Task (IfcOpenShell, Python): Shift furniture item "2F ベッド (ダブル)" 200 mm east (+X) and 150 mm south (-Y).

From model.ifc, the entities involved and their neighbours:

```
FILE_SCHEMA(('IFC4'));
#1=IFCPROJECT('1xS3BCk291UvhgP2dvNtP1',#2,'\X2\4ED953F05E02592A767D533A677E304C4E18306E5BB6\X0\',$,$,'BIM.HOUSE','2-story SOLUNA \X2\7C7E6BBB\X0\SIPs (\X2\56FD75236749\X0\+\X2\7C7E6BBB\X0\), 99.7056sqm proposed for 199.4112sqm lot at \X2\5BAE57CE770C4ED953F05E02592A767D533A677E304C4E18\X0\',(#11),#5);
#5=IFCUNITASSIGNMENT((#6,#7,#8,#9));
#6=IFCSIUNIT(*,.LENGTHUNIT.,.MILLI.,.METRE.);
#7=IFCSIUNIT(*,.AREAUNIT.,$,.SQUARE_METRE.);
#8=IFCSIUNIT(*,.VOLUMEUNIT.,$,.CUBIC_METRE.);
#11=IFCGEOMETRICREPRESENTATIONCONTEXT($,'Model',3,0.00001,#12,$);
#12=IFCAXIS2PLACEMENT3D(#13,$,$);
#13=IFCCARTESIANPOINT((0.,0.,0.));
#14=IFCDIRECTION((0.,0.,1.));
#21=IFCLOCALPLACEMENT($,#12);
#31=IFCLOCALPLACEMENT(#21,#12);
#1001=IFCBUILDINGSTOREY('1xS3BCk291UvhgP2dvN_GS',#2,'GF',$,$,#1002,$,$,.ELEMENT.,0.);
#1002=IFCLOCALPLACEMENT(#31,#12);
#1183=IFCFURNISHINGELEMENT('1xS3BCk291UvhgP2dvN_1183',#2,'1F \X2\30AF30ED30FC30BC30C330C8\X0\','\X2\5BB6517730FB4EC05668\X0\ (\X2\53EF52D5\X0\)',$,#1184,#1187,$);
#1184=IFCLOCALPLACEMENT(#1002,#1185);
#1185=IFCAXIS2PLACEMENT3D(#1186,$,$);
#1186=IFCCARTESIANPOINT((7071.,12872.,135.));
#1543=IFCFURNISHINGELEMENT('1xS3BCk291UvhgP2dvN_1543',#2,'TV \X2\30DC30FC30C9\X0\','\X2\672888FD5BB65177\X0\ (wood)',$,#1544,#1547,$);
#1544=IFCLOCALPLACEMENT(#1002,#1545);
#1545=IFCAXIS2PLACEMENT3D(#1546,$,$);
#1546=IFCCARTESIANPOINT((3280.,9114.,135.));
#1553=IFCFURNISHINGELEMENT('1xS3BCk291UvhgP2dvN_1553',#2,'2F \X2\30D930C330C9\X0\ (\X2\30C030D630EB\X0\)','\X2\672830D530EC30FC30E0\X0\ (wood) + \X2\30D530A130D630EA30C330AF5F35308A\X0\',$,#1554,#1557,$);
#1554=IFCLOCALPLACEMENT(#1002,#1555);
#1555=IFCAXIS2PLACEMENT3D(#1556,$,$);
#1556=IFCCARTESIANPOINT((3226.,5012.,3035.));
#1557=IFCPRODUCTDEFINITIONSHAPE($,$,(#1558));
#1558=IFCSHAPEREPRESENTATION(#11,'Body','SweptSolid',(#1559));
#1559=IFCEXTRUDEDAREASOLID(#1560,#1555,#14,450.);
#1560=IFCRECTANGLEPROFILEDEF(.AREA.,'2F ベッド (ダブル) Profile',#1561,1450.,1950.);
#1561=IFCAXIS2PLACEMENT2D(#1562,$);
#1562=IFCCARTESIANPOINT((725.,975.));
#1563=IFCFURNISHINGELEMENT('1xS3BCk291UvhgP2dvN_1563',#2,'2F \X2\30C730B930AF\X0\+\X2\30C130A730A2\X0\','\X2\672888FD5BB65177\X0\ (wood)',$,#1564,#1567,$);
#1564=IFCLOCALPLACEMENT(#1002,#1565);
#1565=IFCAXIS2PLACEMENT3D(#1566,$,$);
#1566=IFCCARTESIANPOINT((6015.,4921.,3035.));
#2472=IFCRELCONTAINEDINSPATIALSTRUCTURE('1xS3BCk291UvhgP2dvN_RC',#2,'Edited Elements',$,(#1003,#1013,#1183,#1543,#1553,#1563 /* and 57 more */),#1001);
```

```python
import ifcopenshell
import ifcopenshell.api.geometry
import ifcopenshell.util.placement

model = ifcopenshell.open("model.ifc")

item = model.by_guid("1xS3BCk291UvhgP2dvN_1553")
matrix = ifcopenshell.util.placement.get_local_placement(item.ObjectPlacement)
matrix[0, 3] += 200.0
matrix[1, 3] -= 150.0
ifcopenshell.api.geometry.edit_object_placement(model, product=item, matrix=matrix, is_si=False)

print(ifcopenshell.util.placement.get_local_placement(item.ObjectPlacement).round(3) + 0.0)

model.write("model_updated.ifc")
```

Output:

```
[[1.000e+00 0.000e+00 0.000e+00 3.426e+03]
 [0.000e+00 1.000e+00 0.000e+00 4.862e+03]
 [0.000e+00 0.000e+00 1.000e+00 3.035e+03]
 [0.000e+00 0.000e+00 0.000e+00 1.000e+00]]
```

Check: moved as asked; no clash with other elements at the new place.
